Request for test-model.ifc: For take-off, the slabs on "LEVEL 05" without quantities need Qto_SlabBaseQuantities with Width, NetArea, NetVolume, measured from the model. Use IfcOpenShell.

First a look at what the model holds.

```python
import ifcopenshell
import ifcopenshell.util.element
import ifcopenshell.util.unit

model = ifcopenshell.open("test-model.ifc")
print(model.schema)
for unit_type in ("LENGTHUNIT", "AREAUNIT", "VOLUMEUNIT"):
    print(unit_type, ifcopenshell.util.unit.calculate_unit_scale(model, unit_type))
storey = next(s for s in model.by_type("IfcBuildingStorey") if s.Name == "LEVEL 05")
slabs = [e for e in ifcopenshell.util.element.get_decomposition(storey) if e.is_a("IfcSlab")]
for e in sorted(slabs, key=lambda e: e.id()):
    print(e.id(), e.is_a(), e.Name, list(ifcopenshell.util.element.get_psets(e, qtos_only=True)), sep=" | ")
```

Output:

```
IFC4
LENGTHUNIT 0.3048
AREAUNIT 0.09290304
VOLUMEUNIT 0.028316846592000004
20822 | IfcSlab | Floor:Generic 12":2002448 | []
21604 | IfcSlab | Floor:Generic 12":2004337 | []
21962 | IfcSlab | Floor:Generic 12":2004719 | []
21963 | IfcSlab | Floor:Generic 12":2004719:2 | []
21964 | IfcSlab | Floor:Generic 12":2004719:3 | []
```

```python
import ifcopenshell
import ifcopenshell.api.pset
import ifcopenshell.geom
import ifcopenshell.util.element
import ifcopenshell.util.shape
import ifcopenshell.util.unit

model = ifcopenshell.open("test-model.ifc")
unit_scale = ifcopenshell.util.unit.calculate_unit_scale(model)
area_scale = ifcopenshell.util.unit.calculate_unit_scale(model, "AREAUNIT")
volume_scale = ifcopenshell.util.unit.calculate_unit_scale(model, "VOLUMEUNIT")
settings = ifcopenshell.geom.settings()

storey = next(s for s in model.by_type("IfcBuildingStorey") if s.Name == "LEVEL 05")
slabs = [e for e in ifcopenshell.util.element.get_decomposition(storey) if e.is_a("IfcSlab")]

for e in sorted(slabs, key=lambda e: e.id()):
    if ifcopenshell.util.element.get_psets(e, qtos_only=True, should_inherit=False):
        continue
    # Geometry comes back in metres, in the element's own axes.
    shape = ifcopenshell.geom.create_shape(settings, e)
    values = {
        "Width": ifcopenshell.util.shape.get_z(shape.geometry) / unit_scale,
        "NetArea": ifcopenshell.util.shape.get_footprint_area(shape.geometry) / area_scale,
        "NetVolume": ifcopenshell.util.shape.get_volume(shape.geometry) / volume_scale,
    }
    qto = ifcopenshell.api.pset.add_qto(model, product=e, name="Qto_SlabBaseQuantities")
    ifcopenshell.api.pset.edit_qto(model, qto=qto, properties=values)
    print(e.id(), {k: round(v, 3) for k, v in values.items()})

model.write("test-model-out.ifc")
```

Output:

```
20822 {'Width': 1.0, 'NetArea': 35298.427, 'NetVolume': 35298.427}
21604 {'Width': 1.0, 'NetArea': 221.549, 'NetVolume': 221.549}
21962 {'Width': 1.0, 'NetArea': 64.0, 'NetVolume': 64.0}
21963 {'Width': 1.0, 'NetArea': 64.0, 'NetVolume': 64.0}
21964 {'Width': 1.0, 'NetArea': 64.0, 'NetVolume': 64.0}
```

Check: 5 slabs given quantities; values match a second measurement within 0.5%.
